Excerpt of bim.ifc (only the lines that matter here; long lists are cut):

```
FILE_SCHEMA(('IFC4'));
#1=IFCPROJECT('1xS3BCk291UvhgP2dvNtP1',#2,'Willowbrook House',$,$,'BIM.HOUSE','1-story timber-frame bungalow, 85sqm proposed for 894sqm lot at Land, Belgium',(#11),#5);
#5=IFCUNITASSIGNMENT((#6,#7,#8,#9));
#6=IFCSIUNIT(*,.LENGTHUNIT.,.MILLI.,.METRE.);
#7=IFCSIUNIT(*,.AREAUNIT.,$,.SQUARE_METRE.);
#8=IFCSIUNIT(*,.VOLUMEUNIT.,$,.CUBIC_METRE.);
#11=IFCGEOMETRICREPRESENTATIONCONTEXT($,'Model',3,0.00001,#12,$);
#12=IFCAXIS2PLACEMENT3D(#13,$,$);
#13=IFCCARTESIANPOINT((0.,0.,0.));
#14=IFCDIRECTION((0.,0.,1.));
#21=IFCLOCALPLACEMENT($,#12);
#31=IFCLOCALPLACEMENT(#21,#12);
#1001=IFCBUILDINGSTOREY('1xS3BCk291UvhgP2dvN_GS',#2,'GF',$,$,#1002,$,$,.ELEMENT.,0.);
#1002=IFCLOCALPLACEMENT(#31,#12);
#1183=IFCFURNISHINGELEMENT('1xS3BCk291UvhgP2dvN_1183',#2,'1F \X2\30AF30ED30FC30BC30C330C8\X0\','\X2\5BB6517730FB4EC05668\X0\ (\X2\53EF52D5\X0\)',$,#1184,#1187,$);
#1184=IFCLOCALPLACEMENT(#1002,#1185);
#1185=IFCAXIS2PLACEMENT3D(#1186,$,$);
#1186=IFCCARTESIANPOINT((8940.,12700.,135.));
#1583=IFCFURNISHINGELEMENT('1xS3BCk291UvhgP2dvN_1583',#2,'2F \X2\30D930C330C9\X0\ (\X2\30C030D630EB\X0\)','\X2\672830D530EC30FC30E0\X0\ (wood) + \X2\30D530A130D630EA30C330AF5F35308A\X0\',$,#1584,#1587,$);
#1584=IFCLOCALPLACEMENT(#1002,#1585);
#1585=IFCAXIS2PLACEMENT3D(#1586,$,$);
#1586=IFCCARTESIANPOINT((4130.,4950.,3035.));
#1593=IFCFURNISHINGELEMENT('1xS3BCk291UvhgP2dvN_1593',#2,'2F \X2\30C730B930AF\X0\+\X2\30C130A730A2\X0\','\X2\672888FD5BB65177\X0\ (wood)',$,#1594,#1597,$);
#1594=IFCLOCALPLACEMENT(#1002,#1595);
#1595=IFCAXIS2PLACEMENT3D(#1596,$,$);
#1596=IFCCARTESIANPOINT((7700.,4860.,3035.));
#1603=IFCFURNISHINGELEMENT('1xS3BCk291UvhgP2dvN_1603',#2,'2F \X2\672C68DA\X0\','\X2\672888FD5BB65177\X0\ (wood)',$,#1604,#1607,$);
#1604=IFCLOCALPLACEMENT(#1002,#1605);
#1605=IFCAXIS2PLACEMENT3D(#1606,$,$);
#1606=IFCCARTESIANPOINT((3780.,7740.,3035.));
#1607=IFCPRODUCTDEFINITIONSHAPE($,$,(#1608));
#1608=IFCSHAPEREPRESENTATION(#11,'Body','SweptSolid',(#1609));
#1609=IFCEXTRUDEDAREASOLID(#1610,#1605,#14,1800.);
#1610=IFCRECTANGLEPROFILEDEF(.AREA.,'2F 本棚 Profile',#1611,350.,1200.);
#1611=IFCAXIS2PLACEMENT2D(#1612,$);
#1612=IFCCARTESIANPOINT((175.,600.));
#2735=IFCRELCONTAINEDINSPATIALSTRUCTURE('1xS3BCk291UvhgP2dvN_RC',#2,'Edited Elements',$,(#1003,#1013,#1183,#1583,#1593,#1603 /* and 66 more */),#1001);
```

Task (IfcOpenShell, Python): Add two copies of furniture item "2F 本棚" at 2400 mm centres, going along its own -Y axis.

```python
import ifcopenshell
import ifcopenshell.api.geometry
import ifcopenshell.api.root
import ifcopenshell.util.element
import ifcopenshell.util.placement

model = ifcopenshell.open("bim.ifc")


def reuse_history(source, copy):
    """copy_class also copies each property set's owner history, people and application; keep the originals."""
    for rel in copy.IsDefinedBy:
        if rel.is_a("IfcRelDefinesByProperties") and (history := rel.RelatingPropertyDefinition.OwnerHistory):
            rel.RelatingPropertyDefinition.OwnerHistory = source.OwnerHistory
            ifcopenshell.util.element.remove_deep2(model, history)


source = model.by_guid("1xS3BCk291UvhgP2dvN_1603")
base = ifcopenshell.util.placement.get_local_placement(source.ObjectPlacement)
step = -base[:3, 1] * 2400.0

for i in range(1, 3):
    copy = ifcopenshell.api.root.copy_class(model, product=source)
    copy.Representation = ifcopenshell.util.element.copy_deep(
        model, source.Representation, exclude=["IfcGeometricRepresentationContext", "IfcRepresentationMap"]
    )
    reuse_history(source, copy)
    matrix = base.copy()
    matrix[:3, 3] += i * step
    print("added at", matrix[:3, 3].round(3) + 0.0)
    ifcopenshell.api.geometry.edit_object_placement(model, product=copy, matrix=matrix, is_si=False)

model.write("bim_rev.ifc")
```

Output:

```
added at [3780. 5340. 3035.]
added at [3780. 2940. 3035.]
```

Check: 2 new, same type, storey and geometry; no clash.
